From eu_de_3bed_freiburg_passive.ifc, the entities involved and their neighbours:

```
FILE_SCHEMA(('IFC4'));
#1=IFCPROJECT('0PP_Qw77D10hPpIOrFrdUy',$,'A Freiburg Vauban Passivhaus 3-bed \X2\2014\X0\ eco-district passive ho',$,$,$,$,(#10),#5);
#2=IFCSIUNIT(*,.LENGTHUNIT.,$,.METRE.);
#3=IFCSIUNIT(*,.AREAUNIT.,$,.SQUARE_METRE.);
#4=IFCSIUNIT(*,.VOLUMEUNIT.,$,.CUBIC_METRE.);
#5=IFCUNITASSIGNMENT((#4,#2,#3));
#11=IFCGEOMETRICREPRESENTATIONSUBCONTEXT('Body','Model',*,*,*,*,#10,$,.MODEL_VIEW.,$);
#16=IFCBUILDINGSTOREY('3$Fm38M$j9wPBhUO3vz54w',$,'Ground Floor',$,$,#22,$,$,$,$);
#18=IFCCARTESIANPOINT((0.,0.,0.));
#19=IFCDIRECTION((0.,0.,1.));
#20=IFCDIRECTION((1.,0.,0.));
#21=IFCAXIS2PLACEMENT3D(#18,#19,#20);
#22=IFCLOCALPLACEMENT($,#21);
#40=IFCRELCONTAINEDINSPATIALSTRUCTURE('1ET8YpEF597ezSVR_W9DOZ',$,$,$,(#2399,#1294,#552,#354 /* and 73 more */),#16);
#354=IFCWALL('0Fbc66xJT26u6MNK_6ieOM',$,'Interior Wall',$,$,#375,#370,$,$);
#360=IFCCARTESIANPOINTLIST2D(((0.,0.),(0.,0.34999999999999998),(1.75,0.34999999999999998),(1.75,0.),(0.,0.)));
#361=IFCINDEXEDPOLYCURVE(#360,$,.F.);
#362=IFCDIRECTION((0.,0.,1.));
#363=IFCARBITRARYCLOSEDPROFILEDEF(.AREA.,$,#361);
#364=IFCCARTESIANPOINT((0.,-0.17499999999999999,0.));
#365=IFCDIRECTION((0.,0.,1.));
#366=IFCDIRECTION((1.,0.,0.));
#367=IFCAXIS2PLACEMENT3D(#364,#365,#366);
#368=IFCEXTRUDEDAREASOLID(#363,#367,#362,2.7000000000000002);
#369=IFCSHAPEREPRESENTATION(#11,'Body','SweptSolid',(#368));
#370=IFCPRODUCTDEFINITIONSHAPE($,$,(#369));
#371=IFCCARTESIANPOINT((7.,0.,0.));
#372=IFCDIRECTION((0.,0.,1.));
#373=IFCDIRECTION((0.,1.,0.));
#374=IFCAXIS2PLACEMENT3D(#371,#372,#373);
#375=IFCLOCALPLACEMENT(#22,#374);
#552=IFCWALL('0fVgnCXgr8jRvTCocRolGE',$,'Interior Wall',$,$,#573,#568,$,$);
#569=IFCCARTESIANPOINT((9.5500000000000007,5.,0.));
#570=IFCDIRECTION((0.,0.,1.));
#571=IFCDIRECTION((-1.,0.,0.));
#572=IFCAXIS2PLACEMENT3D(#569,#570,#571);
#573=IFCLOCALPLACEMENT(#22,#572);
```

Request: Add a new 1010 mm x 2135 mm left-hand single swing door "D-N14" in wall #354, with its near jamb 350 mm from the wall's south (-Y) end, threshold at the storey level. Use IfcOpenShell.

```python
import numpy as np
import ifcopenshell
import ifcopenshell.api.feature
import ifcopenshell.api.geometry
import ifcopenshell.api.root
import ifcopenshell.api.spatial
import ifcopenshell.geom
import ifcopenshell.util.element
import ifcopenshell.util.placement
import ifcopenshell.util.representation
import ifcopenshell.util.shape
import ifcopenshell.util.unit

model = ifcopenshell.open("eu_de_3bed_freiburg_passive.ifc")
unit_scale = ifcopenshell.util.unit.calculate_unit_scale(model)
settings = ifcopenshell.geom.settings()


def volume(element):
    """Net volume in cubic metres, openings subtracted."""
    shape = ifcopenshell.geom.create_shape(settings, element)
    return ifcopenshell.util.shape.get_volume(shape.geometry)


wall = model.by_id(354)
storey = ifcopenshell.util.element.get_container(wall, ifc_class="IfcBuildingStorey")
context = ifcopenshell.util.representation.get_context(model, "Model", "Body", "MODEL_VIEW")
before = volume(wall)

width, height, from_end, sill = 1.01, 2.135, 0.35, 0.0  # metres

# The wall runs along its own X axis, and the end named is its -X end.
wall_shape = ifcopenshell.geom.create_shape(settings, wall)
x, y, z = ifcopenshell.util.shape.get_vertices(wall_shape.geometry).T
start = x.min() + from_end
face, thickness = float(y.min()), float(y.max() - y.min())
wall_matrix = ifcopenshell.util.placement.get_local_placement(wall.ObjectPlacement)
level = ifcopenshell.util.placement.get_local_placement(storey.ObjectPlacement)[2, 3]


def in_wall(x, y):
    """Placement at x, y metres in the wall's axes, at sill height."""
    matrix = wall_matrix.copy()
    matrix[:, 3] = wall_matrix @ np.array([x / unit_scale, y / unit_scale, 0.0, 1.0])
    matrix[2, 3] = level + sill / unit_scale
    return matrix


# Opening: a box that overshoots both wall faces by 50 mm.
opening = ifcopenshell.api.root.create_entity(model, ifc_class="IfcOpeningElement", predefined_type="OPENING")
box = ifcopenshell.api.geometry.add_wall_representation(
    model, context=context, length=width, height=height, thickness=thickness + 0.1
)
ifcopenshell.api.geometry.assign_representation(model, product=opening, representation=box)
ifcopenshell.api.geometry.edit_object_placement(model, product=opening, matrix=in_wall(start, face - 0.05), is_si=False)
ifcopenshell.api.feature.add_feature(model, feature=opening, element=wall)

door = ifcopenshell.api.root.create_entity(model, ifc_class="IfcDoor", name="D-N14", predefined_type="DOOR")
door.OverallWidth, door.OverallHeight = width / unit_scale, height / unit_scale
door.OperationType = "SINGLE_SWING_LEFT"
body = ifcopenshell.api.geometry.add_door_representation(
    model,
    context=context,
    overall_width=door.OverallWidth,
    overall_height=door.OverallHeight,
    operation_type="SINGLE_SWING_LEFT",
    lining_properties={"LiningDepth": thickness / unit_scale, "ThresholdDepth": thickness / unit_scale},
)
ifcopenshell.api.geometry.assign_representation(model, product=door, representation=body)
ifcopenshell.api.spatial.assign_container(model, products=[door], relating_structure=storey)
ifcopenshell.api.feature.add_filling(model, opening=opening, element=door)

# The lining spans the wall, so the door starts at the wall face.
ifcopenshell.api.geometry.edit_object_placement(model, product=door, matrix=in_wall(start, face), is_si=False)

after = volume(wall)

print(f"wall volume {before:.3f} -> {after:.3f} m3")

model.write("eu_de_3bed_freiburg_passive_updated.ifc")
```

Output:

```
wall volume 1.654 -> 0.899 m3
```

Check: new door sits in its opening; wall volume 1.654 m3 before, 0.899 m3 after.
